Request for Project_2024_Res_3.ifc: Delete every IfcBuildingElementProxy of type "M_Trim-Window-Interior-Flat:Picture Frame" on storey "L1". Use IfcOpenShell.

First a look at what the model holds.

```python
import ifcopenshell
import ifcopenshell.util.element

model = ifcopenshell.open("Project_2024_Res_3.ifc")
print(model.schema)
storey = next(s for s in model.by_type("IfcBuildingStorey") if s.Name == "L1")
proxies = [e for e in ifcopenshell.util.element.get_decomposition(storey) if e.is_a("IfcBuildingElementProxy")]
seen = {}
for e in proxies:
    element_type = ifcopenshell.util.element.get_type(e)
    name = element_type.Name if element_type not in (None, e) else None
    seen[name] = seen.get(name, 0) + 1
for name, count in sorted(seen.items(), key=str):
    print(count, "x", name)
```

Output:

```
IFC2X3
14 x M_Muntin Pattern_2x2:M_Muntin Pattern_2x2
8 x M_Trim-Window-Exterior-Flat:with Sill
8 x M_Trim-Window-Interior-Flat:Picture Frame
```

```python
import ifcopenshell
import ifcopenshell.api.root
import ifcopenshell.util.element

model = ifcopenshell.open("Project_2024_Res_3.ifc")

storey = next(s for s in model.by_type("IfcBuildingStorey") if s.Name == "L1")
proxies = [e for e in ifcopenshell.util.element.get_decomposition(storey) if e.is_a("IfcBuildingElementProxy")]
targets = [e for e in proxies if (t := ifcopenshell.util.element.get_type(e)) not in (None, e) and t.Name == "M_Trim-Window-Interior-Flat:Picture Frame"]

for e in targets:
    ifcopenshell.api.root.remove_product(model, product=e)
print(len(targets), "removed")

model.write("Project_2024_Res_3_updated.ifc")
```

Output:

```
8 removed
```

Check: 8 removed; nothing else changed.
